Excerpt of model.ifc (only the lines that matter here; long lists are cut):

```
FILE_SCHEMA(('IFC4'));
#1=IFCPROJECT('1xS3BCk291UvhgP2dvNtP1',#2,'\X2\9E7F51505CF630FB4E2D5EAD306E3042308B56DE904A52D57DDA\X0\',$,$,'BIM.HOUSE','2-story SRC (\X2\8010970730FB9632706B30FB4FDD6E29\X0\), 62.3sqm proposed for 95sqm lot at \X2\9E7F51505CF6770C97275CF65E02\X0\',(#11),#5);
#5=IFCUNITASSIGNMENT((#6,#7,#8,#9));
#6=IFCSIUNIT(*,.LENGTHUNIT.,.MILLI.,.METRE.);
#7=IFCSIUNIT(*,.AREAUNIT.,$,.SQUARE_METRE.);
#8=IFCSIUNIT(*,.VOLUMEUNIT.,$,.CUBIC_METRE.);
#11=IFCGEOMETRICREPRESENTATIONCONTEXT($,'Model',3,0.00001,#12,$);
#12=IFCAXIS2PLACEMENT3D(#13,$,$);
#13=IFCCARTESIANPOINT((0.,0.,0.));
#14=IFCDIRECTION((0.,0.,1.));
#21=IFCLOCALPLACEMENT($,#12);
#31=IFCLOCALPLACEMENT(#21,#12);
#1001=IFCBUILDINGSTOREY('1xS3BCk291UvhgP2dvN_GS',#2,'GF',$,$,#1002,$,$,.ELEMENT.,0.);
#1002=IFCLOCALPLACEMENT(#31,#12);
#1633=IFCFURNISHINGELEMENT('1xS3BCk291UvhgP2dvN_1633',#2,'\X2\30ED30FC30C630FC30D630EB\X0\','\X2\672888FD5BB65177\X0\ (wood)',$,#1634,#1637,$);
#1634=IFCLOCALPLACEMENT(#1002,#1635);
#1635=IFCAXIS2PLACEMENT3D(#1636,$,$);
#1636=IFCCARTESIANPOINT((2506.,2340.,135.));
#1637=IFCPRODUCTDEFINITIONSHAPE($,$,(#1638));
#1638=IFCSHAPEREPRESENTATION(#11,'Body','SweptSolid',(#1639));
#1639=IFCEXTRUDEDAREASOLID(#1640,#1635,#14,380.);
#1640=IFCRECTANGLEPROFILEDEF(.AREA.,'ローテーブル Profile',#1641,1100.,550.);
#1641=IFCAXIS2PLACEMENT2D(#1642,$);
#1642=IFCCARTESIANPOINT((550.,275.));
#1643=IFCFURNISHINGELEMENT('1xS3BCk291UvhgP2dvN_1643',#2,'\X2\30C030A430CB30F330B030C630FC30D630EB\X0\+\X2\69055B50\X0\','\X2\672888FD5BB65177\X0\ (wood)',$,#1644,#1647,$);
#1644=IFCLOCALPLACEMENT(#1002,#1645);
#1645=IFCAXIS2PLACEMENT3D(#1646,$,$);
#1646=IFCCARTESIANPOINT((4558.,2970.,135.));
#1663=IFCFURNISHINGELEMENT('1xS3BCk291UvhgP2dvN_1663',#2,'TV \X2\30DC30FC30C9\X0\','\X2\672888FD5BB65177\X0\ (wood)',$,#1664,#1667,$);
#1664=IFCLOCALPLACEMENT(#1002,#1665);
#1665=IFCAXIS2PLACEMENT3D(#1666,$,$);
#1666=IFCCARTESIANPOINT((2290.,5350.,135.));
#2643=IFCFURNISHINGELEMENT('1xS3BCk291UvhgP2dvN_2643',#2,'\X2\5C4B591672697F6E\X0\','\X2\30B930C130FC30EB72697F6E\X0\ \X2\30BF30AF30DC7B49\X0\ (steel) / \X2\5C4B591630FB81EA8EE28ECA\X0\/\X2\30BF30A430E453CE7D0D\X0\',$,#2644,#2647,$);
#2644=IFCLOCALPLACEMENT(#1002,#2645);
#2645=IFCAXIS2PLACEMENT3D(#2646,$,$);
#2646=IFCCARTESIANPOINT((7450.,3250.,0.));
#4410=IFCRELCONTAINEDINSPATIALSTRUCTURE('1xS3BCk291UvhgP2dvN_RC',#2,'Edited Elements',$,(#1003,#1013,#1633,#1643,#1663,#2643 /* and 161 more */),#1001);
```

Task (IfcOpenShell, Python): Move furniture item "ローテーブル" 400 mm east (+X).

```python
import ifcopenshell
import ifcopenshell.api.geometry
import ifcopenshell.util.placement
import ifcopenshell.util.unit

model = ifcopenshell.open("model.ifc")
unit_scale = ifcopenshell.util.unit.calculate_unit_scale(model)

item = model.by_guid("1xS3BCk291UvhgP2dvN_1633")
matrix = ifcopenshell.util.placement.get_local_placement(item.ObjectPlacement)
matrix[0, 3] += 0.4 / unit_scale
ifcopenshell.api.geometry.edit_object_placement(model, product=item, matrix=matrix, is_si=False)

print(ifcopenshell.util.placement.get_local_placement(item.ObjectPlacement).round(3) + 0.0)

model.write("model-out.ifc")
```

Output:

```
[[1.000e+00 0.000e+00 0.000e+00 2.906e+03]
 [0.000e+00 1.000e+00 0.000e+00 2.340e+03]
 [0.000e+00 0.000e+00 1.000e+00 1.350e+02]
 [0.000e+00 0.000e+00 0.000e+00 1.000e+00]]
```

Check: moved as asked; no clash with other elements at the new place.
